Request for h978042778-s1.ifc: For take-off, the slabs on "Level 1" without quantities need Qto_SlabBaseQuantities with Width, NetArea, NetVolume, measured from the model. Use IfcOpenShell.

First a look at what the model holds.

```python
import ifcopenshell
import ifcopenshell.util.element
import ifcopenshell.util.unit

model = ifcopenshell.open("h978042778-s1.ifc")
print(model.schema)
for unit_type in ("LENGTHUNIT", "AREAUNIT", "VOLUMEUNIT"):
    print(unit_type, ifcopenshell.util.unit.calculate_unit_scale(model, unit_type))
storey = next(s for s in model.by_type("IfcBuildingStorey") if s.Name == "Level 1")
slabs = [e for e in ifcopenshell.util.element.get_decomposition(storey) if e.is_a("IfcSlab")]
for e in sorted(slabs, key=lambda e: e.id()):
    print(e.id(), e.is_a(), e.Name, list(ifcopenshell.util.element.get_psets(e, qtos_only=True)), sep=" | ")
```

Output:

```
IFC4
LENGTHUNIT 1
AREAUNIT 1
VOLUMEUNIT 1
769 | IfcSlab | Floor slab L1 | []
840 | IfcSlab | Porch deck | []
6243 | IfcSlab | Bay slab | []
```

```python
import ifcopenshell
import ifcopenshell.api.pset
import ifcopenshell.geom
import ifcopenshell.util.element
import ifcopenshell.util.shape
import ifcopenshell.util.unit

model = ifcopenshell.open("h978042778-s1.ifc")
unit_scale = ifcopenshell.util.unit.calculate_unit_scale(model)
area_scale = ifcopenshell.util.unit.calculate_unit_scale(model, "AREAUNIT")
volume_scale = ifcopenshell.util.unit.calculate_unit_scale(model, "VOLUMEUNIT")
settings = ifcopenshell.geom.settings()

storey = next(s for s in model.by_type("IfcBuildingStorey") if s.Name == "Level 1")
slabs = [e for e in ifcopenshell.util.element.get_decomposition(storey) if e.is_a("IfcSlab")]

for e in sorted(slabs, key=lambda e: e.id()):
    if ifcopenshell.util.element.get_psets(e, qtos_only=True, should_inherit=False):
        continue
    # Geometry comes back in metres, in the element's own axes.
    shape = ifcopenshell.geom.create_shape(settings, e)
    values = {
        "Width": ifcopenshell.util.shape.get_z(shape.geometry) / unit_scale,
        "NetArea": ifcopenshell.util.shape.get_footprint_area(shape.geometry) / area_scale,
        "NetVolume": ifcopenshell.util.shape.get_volume(shape.geometry) / volume_scale,
    }
    qto = ifcopenshell.api.pset.add_qto(model, product=e, name="Qto_SlabBaseQuantities")
    ifcopenshell.api.pset.edit_qto(model, qto=qto, properties=values)
    print(e.id(), {k: round(v, 3) for k, v in values.items()})

model.write("h978042778-s1_updated.ifc")
```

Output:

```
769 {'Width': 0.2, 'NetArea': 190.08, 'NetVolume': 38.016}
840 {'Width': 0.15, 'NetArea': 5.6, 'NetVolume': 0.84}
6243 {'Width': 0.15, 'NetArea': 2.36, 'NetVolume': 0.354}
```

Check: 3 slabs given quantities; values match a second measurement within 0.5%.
